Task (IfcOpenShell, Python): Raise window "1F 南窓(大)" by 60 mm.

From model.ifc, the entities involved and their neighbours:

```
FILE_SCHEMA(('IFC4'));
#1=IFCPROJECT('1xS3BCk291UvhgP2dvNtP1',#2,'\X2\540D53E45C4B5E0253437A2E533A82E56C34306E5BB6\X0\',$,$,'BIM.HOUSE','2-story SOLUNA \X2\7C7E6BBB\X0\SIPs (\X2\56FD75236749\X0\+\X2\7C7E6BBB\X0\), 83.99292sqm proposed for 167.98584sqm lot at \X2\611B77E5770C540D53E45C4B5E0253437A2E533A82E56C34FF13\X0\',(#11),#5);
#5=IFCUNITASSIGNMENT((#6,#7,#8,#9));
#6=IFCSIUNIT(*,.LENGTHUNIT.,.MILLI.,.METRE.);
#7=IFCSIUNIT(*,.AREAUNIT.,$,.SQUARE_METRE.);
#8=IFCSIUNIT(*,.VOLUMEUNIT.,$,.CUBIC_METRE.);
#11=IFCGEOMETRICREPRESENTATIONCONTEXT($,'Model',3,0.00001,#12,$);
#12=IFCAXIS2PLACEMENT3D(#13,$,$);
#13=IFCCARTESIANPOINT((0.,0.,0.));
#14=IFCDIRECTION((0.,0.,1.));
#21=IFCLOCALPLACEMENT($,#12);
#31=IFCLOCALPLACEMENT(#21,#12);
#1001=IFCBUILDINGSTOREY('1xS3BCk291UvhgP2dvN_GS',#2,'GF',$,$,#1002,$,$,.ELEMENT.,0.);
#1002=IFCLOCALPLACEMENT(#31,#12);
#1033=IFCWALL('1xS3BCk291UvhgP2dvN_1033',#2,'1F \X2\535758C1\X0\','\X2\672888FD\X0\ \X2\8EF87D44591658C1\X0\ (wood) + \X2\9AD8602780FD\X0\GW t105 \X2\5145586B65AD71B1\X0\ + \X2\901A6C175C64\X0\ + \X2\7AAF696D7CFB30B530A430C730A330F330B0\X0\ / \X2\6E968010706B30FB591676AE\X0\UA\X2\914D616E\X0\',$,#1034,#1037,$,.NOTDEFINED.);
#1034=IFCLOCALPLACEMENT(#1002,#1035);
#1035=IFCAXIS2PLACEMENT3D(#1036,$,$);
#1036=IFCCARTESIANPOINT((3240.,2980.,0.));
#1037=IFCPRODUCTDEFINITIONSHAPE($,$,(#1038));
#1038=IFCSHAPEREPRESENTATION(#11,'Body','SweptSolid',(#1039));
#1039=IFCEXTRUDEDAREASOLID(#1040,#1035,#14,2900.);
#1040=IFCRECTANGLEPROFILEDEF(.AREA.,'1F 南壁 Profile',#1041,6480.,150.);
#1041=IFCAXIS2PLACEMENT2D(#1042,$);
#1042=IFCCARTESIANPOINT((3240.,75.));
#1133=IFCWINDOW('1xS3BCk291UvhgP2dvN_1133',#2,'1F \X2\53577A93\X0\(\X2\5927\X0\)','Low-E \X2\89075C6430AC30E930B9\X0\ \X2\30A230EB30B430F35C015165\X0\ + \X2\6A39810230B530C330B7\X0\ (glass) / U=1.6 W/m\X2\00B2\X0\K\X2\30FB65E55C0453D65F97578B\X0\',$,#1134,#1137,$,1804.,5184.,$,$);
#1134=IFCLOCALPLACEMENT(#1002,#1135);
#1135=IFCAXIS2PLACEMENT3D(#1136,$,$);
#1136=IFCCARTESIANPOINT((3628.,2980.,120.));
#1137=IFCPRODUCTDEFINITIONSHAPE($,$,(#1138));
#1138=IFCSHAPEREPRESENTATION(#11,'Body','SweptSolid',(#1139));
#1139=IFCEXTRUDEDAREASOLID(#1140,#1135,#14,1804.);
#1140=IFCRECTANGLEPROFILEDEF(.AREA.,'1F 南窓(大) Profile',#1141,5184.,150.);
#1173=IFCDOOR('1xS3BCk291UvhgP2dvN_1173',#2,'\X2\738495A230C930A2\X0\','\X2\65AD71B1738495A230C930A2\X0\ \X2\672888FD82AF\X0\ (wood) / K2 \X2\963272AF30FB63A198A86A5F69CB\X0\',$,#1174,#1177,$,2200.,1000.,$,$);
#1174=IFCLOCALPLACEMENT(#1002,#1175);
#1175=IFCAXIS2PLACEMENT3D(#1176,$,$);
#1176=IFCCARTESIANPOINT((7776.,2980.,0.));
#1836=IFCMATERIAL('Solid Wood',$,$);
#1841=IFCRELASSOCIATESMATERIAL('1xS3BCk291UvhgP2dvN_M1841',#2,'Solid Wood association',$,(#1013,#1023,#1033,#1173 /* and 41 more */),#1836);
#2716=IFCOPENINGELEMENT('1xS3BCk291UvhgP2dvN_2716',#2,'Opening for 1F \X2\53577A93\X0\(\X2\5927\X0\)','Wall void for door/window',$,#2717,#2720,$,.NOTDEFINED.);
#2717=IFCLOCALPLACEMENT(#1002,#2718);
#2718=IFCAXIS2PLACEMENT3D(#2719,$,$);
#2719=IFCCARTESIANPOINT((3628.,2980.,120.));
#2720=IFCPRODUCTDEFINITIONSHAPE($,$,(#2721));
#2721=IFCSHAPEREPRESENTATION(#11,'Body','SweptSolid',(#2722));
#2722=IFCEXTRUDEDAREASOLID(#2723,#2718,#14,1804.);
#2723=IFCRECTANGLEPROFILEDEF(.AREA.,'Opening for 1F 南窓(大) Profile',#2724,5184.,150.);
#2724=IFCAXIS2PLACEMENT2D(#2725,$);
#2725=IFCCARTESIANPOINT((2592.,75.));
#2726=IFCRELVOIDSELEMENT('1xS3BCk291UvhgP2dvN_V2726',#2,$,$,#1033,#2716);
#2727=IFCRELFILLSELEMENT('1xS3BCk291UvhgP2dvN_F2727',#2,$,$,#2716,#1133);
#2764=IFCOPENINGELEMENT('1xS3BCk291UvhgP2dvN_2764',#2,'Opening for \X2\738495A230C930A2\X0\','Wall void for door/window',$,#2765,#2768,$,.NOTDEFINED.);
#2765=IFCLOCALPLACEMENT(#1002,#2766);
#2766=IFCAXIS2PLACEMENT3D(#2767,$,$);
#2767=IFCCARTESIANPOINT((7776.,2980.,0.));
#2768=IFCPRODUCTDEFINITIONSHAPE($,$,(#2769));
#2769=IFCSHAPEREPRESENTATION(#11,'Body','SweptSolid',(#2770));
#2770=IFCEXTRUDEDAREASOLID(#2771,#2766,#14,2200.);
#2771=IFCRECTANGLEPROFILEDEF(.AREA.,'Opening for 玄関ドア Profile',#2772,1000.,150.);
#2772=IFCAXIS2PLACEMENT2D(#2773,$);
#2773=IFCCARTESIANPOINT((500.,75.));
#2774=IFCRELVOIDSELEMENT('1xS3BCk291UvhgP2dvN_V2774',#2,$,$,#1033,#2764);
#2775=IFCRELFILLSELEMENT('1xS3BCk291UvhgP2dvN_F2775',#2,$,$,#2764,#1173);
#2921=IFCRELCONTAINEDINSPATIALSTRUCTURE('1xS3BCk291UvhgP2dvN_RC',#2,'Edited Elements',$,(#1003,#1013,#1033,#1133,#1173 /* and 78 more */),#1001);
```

```python
import numpy as np
import ifcopenshell
import ifcopenshell.api.geometry
import ifcopenshell.util.placement
import ifcopenshell.util.unit

model = ifcopenshell.open("model.ifc")
unit_scale = ifcopenshell.util.unit.calculate_unit_scale(model)

window = model.by_guid("1xS3BCk291UvhgP2dvN_1133")
opening = window.FillsVoids[0].RelatingOpeningElement
dz = 60.0

shift = np.array([0.0, 0.0, dz])
# The window is not placed relative to its opening, so move both.
for product in (opening, window):
    matrix = ifcopenshell.util.placement.get_local_placement(product.ObjectPlacement)
    matrix[:3, 3] += shift
    ifcopenshell.api.geometry.edit_object_placement(model, product=product, matrix=matrix, is_si=False)

print(f"moved by {dz * unit_scale:+.3f} m")

model.write("model_updated.ifc")
```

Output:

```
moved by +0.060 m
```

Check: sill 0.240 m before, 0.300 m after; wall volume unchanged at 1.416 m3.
